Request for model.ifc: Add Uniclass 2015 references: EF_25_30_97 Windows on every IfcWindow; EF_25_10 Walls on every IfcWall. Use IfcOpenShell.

First a look at what the model holds.

```python
import ifcopenshell

model = ifcopenshell.open("model.ifc")
print(model.schema)
print("classifications:", [c.Name for c in model.by_type("IfcClassification")])
for ifc_class in ("IfcDoor", "IfcRoof", "IfcStair", "IfcWall", "IfcWindow"):
    print(ifc_class, len(model.by_type(ifc_class)))
```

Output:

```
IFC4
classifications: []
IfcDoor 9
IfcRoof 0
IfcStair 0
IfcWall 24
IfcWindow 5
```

```python
import ifcopenshell
import ifcopenshell.api.classification

model = ifcopenshell.open("model.ifc")

system = ifcopenshell.api.classification.add_classification(model, classification="Uniclass 2015")

codes = {
    "IfcWindow": ("EF_25_30_97", "Windows"),
    "IfcWall": ("EF_25_10", "Walls"),
}
for ifc_class, (code, name) in codes.items():
    products = model.by_type(ifc_class)
    ifcopenshell.api.classification.add_reference(
        model, products=products, classification=system, identification=code, name=name
    )
    print(code, len(products))

model.write("model-out.ifc")
```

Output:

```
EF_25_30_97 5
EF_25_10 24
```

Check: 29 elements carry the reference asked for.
